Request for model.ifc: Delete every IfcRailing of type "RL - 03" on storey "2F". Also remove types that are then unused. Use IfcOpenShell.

First a look at what the model holds.

```python
import ifcopenshell
import ifcopenshell.util.element

model = ifcopenshell.open("model.ifc")
print(model.schema)
storey = next(s for s in model.by_type("IfcBuildingStorey") if s.Name == "2F")
railings = [e for e in ifcopenshell.util.element.get_decomposition(storey) if e.is_a("IfcRailing")]
seen = {}
for e in railings:
    element_type = ifcopenshell.util.element.get_type(e)
    name = element_type.Name if element_type not in (None, e) else None
    seen[name] = seen.get(name, 0) + 1
for name, count in sorted(seen.items(), key=str):
    print(count, "x", name)
```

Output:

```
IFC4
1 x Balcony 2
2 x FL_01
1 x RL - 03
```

```python
import ifcopenshell
import ifcopenshell.api.root
import ifcopenshell.util.element

model = ifcopenshell.open("model.ifc")

storey = next(s for s in model.by_type("IfcBuildingStorey") if s.Name == "2F")
railings = [e for e in ifcopenshell.util.element.get_decomposition(storey) if e.is_a("IfcRailing")]
targets = [e for e in railings if (t := ifcopenshell.util.element.get_type(e)) not in (None, e) and t.Name == "RL - 03"]
types = {ifcopenshell.util.element.get_type(e) for e in targets} - {None, *targets}

for e in targets:
    ifcopenshell.api.root.remove_product(model, product=e)
print(len(targets), "removed")

unused = [t for t in types if not ifcopenshell.util.element.get_types(t)]
for t in unused:
    ifcopenshell.api.root.remove_product(model, product=t)
print(len(unused), "unused types removed")

model.write("model_rev.ifc")
```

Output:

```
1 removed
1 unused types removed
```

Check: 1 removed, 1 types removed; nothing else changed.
